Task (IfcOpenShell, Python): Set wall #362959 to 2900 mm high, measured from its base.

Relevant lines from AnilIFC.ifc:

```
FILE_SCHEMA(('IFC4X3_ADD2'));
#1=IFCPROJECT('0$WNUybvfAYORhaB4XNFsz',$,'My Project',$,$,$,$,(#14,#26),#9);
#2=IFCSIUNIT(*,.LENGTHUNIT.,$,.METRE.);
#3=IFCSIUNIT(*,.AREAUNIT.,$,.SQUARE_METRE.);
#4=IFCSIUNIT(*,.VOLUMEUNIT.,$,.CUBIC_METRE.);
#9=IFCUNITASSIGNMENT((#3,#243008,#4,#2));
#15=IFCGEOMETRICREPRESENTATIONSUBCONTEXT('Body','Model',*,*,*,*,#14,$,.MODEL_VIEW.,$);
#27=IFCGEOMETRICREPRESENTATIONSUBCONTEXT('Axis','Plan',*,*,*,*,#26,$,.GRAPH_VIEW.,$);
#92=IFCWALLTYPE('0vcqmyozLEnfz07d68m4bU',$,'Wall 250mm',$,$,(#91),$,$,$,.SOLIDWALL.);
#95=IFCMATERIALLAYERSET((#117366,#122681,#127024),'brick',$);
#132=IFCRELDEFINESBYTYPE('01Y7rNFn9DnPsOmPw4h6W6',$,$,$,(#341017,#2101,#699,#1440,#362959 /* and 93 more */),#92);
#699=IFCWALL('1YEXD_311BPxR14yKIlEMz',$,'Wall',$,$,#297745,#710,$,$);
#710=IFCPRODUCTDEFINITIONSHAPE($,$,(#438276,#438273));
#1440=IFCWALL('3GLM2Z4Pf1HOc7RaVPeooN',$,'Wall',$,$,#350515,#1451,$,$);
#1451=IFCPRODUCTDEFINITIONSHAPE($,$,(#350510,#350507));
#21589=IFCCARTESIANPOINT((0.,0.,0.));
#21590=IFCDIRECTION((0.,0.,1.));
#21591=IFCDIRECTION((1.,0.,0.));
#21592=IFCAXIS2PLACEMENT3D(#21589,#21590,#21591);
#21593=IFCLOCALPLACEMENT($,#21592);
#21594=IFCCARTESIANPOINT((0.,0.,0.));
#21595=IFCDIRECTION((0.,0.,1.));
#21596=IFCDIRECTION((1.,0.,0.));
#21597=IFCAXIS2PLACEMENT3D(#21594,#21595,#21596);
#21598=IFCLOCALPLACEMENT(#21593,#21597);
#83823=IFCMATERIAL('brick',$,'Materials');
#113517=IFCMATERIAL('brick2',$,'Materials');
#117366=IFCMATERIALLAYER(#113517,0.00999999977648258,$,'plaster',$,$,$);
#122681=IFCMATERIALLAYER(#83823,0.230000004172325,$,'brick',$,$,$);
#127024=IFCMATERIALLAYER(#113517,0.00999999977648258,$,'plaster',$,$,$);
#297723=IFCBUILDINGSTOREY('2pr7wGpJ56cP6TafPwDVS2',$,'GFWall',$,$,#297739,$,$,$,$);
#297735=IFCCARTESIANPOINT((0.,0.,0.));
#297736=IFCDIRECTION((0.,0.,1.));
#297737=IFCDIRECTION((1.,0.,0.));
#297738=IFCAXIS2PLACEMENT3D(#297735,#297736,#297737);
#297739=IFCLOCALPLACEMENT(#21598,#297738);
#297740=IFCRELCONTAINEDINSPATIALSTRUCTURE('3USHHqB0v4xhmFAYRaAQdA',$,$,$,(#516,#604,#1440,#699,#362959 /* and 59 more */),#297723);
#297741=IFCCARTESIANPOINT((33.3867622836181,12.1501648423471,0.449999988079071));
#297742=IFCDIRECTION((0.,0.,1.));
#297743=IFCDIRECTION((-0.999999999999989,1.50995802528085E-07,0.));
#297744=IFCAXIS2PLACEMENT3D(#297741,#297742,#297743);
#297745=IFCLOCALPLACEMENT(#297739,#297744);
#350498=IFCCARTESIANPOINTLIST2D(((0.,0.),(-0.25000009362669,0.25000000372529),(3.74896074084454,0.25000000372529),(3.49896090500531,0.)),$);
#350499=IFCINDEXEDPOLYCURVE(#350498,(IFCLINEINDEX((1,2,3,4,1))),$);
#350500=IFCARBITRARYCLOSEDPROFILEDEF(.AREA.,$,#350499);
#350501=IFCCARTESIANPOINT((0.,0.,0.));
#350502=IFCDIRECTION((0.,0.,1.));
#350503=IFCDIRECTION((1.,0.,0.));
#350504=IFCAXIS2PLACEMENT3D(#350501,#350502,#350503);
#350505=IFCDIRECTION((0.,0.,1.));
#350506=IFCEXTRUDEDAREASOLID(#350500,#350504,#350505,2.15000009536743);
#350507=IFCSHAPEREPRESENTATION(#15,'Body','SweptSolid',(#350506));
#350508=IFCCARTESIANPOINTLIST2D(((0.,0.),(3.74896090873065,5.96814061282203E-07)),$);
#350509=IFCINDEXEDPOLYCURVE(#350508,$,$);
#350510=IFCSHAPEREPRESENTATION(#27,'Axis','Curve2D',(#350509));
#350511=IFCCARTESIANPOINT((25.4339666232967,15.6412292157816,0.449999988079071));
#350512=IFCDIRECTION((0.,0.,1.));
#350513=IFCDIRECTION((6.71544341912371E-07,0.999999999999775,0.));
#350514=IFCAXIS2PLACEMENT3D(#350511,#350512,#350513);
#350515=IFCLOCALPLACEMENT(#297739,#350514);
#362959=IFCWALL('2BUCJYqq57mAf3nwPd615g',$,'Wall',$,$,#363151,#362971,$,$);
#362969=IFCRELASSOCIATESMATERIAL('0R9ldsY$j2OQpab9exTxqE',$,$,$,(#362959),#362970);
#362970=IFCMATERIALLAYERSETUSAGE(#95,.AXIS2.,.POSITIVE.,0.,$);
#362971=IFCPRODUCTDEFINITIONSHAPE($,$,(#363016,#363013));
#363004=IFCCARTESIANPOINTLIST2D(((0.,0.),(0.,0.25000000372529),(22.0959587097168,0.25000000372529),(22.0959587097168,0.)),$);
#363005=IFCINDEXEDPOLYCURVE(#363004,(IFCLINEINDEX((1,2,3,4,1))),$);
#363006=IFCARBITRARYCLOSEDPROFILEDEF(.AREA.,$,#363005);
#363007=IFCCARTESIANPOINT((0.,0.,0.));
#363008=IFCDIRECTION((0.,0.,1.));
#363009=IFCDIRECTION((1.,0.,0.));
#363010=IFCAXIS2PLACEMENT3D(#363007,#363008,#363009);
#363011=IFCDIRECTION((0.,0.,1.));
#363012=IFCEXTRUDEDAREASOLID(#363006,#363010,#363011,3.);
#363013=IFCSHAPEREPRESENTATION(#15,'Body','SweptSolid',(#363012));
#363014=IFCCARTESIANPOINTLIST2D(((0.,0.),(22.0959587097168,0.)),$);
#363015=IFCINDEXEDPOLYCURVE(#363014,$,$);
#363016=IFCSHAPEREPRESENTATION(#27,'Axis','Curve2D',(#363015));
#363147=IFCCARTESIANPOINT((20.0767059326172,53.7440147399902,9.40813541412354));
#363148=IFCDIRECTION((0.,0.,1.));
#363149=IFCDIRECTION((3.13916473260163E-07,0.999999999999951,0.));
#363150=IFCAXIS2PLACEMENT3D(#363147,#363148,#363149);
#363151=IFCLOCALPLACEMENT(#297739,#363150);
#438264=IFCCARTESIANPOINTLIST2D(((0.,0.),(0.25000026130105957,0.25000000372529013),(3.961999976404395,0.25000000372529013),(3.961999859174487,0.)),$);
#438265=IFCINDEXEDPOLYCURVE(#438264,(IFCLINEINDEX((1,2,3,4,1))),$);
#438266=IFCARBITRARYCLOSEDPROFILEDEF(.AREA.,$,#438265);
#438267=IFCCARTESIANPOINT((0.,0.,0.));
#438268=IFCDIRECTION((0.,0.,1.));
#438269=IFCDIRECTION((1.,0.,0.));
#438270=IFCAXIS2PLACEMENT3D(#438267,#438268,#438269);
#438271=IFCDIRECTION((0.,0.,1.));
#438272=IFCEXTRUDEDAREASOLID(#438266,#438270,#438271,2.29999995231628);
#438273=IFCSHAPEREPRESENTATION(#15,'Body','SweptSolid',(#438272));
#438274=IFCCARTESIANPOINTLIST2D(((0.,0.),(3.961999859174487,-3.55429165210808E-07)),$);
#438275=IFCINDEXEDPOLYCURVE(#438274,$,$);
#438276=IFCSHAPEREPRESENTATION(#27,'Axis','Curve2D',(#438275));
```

```python
import ifcopenshell
import ifcopenshell.geom
import ifcopenshell.util.representation
import ifcopenshell.util.shape
import ifcopenshell.util.unit

model = ifcopenshell.open("AnilIFC.ifc")
unit_scale = ifcopenshell.util.unit.calculate_unit_scale(model)
settings = ifcopenshell.geom.settings()


def volume(element):
    """Net volume in cubic metres, openings subtracted."""
    shape = ifcopenshell.geom.create_shape(settings, element)
    return ifcopenshell.util.shape.get_volume(shape.geometry)


wall = model.by_guid("2BUCJYqq57mAf3nwPd615g")
before = volume(wall)

body = ifcopenshell.util.representation.get_representation(wall, "Model", "Body")
solid = body.Items[0]
old_height = solid.Depth
solid.Depth = 2.9 / unit_scale
after = volume(wall)

print(f"height {old_height:g} -> {solid.Depth:g}, volume {before:.3f} -> {after:.3f} m3")

model.write("AnilIFC-out.ifc")
```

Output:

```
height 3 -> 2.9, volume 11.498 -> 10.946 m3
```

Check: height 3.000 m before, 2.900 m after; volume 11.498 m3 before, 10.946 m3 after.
